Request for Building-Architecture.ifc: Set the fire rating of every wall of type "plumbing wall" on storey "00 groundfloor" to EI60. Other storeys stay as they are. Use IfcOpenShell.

First a look at what the model holds.

```python
import ifcopenshell
import ifcopenshell.util.element

model = ifcopenshell.open("Building-Architecture.ifc")
print(model.schema)
storey = next(s for s in model.by_type("IfcBuildingStorey") if s.Name == "00 groundfloor")
walls = [e for e in ifcopenshell.util.element.get_decomposition(storey) if e.is_a("IfcWall")]
seen = {}
for e in walls:
    element_type = ifcopenshell.util.element.get_type(e)
    key = (element_type.Name if element_type != e and element_type else None, ifcopenshell.util.element.get_pset(e, "Pset_WallCommon", "FireRating"))
    seen[key] = seen.get(key, 0) + 1
for (name, value), count in sorted(seen.items(), key=str):
    print(count, "x", name, "|", value)
```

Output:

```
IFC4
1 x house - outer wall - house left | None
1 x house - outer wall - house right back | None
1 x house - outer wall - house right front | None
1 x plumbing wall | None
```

```python
import ifcopenshell
import ifcopenshell.api.pset
import ifcopenshell.util.element

model = ifcopenshell.open("Building-Architecture.ifc")

storey = next(s for s in model.by_type("IfcBuildingStorey") if s.Name == "00 groundfloor")
walls = [e for e in ifcopenshell.util.element.get_decomposition(storey) if e.is_a("IfcWall")]

count = 0
for e in walls:
    element_type = ifcopenshell.util.element.get_type(e)
    if element_type in (None, e) or element_type.Name != "plumbing wall":
        continue
    # add_pset returns the element's existing set when there is one.
    pset = ifcopenshell.api.pset.add_pset(model, product=e, name="Pset_WallCommon")
    ifcopenshell.api.pset.edit_pset(model, pset=pset, properties={"FireRating": "EI60"})
    count += 1

print(count, "walls updated")

model.write("Building-Architecture_updated.ifc")
```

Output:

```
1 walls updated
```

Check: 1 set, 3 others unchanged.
